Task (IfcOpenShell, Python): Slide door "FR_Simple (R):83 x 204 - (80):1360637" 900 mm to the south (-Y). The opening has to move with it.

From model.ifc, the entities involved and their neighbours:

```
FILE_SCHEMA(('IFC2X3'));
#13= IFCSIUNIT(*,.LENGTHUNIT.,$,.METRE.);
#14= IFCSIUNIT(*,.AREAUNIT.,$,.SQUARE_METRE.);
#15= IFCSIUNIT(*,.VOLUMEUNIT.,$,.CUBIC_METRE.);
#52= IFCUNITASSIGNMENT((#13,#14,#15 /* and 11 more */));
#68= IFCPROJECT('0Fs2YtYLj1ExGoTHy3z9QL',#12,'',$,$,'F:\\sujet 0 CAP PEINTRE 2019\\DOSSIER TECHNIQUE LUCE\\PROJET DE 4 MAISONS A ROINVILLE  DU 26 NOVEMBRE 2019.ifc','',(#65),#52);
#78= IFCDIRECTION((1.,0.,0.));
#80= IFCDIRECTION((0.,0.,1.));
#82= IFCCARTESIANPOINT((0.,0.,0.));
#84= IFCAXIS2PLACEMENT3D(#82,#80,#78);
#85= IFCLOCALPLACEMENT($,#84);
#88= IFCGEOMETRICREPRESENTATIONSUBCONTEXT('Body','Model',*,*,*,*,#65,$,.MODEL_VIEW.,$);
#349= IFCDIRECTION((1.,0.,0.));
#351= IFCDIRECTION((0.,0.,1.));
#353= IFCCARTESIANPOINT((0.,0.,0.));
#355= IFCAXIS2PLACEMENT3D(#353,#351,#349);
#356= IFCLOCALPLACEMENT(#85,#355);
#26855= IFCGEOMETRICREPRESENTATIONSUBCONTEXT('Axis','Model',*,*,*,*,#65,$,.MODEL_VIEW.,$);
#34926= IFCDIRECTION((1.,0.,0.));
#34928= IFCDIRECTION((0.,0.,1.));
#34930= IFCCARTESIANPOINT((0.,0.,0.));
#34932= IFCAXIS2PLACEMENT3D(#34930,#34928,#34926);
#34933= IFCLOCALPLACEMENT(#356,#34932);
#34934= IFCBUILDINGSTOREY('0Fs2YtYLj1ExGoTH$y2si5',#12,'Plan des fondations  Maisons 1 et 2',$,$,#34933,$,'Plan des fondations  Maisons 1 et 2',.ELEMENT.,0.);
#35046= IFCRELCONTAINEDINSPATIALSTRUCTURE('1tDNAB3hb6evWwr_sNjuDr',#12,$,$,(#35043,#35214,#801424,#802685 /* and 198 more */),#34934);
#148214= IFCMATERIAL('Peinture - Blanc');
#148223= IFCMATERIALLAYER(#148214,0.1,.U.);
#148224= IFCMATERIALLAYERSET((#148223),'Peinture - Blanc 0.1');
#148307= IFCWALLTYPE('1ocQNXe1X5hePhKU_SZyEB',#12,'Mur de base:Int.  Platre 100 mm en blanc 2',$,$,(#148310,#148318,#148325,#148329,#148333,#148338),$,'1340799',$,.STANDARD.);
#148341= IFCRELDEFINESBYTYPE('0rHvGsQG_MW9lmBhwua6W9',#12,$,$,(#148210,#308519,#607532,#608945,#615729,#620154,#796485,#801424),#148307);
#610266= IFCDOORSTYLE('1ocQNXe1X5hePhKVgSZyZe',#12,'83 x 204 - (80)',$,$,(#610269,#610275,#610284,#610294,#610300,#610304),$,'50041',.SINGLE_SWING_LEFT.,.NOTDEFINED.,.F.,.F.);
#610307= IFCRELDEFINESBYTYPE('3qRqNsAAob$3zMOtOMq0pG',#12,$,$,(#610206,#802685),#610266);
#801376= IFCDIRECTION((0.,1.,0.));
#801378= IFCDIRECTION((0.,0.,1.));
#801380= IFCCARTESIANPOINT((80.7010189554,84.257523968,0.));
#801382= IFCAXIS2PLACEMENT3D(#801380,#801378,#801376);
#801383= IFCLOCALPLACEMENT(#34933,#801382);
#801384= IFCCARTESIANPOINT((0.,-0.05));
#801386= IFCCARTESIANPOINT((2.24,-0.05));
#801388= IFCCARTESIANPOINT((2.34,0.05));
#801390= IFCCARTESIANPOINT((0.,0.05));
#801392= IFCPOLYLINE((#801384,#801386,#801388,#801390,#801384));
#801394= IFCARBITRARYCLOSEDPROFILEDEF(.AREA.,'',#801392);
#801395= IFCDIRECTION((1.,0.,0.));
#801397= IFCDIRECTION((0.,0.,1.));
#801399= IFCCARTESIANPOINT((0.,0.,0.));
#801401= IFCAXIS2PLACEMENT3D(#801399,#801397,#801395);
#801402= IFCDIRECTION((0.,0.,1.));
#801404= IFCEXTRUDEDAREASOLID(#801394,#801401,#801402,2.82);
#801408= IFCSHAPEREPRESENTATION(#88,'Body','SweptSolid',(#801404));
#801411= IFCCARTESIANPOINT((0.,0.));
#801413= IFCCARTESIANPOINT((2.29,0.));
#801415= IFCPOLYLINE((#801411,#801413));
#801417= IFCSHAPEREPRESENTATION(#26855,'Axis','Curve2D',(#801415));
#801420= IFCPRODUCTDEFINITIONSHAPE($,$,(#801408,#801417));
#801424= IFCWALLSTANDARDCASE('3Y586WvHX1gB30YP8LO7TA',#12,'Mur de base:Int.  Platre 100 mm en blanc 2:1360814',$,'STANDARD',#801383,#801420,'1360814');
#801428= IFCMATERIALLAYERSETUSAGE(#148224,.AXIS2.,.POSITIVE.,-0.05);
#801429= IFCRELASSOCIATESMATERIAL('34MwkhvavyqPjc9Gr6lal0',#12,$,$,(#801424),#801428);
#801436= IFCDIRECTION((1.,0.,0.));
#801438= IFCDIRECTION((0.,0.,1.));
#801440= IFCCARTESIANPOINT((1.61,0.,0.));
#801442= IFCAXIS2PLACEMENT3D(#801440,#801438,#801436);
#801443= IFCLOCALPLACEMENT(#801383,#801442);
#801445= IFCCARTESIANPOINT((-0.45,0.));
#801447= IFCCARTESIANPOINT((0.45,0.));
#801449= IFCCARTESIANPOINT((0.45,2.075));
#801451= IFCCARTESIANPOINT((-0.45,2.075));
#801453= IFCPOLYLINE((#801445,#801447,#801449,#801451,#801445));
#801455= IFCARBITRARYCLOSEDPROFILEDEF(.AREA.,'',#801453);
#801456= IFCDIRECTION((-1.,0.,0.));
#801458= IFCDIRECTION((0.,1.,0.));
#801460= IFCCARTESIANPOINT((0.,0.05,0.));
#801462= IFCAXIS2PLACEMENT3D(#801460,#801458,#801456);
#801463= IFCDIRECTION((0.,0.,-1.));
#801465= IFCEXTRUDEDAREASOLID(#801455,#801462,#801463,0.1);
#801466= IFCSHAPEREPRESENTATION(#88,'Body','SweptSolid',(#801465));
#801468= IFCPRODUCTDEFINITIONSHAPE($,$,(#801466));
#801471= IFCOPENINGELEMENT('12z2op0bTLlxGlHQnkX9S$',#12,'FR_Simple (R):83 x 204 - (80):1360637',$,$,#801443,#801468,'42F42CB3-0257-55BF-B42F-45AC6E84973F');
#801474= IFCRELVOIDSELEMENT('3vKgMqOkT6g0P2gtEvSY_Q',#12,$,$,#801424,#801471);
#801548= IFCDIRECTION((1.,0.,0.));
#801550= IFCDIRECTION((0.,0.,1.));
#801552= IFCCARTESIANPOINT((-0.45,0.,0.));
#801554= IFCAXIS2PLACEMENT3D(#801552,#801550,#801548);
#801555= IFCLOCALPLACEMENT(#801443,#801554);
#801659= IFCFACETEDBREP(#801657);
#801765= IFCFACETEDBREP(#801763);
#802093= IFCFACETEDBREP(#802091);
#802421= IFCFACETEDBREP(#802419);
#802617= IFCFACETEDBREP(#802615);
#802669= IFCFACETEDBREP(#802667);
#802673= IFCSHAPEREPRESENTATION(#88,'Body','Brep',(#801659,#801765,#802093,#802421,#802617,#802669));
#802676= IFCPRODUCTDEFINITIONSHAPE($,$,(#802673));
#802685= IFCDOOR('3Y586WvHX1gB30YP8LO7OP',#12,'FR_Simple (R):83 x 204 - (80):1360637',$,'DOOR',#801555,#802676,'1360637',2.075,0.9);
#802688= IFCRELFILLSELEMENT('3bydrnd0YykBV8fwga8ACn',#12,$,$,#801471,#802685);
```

```python
import ifcopenshell
import ifcopenshell.api.geometry
import ifcopenshell.util.placement

model = ifcopenshell.open("model.ifc")

door = model.by_id(802685)
opening = door.FillsVoids[0].RelatingOpeningElement
wall = opening.VoidsElements[0].RelatingBuildingElement

wall_matrix = ifcopenshell.util.placement.get_local_placement(wall.ObjectPlacement)
shift = wall_matrix[:3, 0] * -0.9
before = ifcopenshell.util.placement.get_local_placement(door.ObjectPlacement)[:3, 3].copy()

# The door is placed relative to its opening, so it follows when the opening moves.
matrix = ifcopenshell.util.placement.get_local_placement(opening.ObjectPlacement)
matrix[:3, 3] += shift
ifcopenshell.api.geometry.edit_object_placement(
    model, product=opening, matrix=matrix, is_si=False, should_transform_children=True
)

after = ifcopenshell.util.placement.get_local_placement(door.ObjectPlacement)[:3, 3]
print("door moved by", (after - before).round(3) + 0.0)

model.write("model_rev.ifc")
```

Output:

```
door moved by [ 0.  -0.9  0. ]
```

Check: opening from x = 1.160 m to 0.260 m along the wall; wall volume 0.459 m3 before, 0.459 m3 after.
